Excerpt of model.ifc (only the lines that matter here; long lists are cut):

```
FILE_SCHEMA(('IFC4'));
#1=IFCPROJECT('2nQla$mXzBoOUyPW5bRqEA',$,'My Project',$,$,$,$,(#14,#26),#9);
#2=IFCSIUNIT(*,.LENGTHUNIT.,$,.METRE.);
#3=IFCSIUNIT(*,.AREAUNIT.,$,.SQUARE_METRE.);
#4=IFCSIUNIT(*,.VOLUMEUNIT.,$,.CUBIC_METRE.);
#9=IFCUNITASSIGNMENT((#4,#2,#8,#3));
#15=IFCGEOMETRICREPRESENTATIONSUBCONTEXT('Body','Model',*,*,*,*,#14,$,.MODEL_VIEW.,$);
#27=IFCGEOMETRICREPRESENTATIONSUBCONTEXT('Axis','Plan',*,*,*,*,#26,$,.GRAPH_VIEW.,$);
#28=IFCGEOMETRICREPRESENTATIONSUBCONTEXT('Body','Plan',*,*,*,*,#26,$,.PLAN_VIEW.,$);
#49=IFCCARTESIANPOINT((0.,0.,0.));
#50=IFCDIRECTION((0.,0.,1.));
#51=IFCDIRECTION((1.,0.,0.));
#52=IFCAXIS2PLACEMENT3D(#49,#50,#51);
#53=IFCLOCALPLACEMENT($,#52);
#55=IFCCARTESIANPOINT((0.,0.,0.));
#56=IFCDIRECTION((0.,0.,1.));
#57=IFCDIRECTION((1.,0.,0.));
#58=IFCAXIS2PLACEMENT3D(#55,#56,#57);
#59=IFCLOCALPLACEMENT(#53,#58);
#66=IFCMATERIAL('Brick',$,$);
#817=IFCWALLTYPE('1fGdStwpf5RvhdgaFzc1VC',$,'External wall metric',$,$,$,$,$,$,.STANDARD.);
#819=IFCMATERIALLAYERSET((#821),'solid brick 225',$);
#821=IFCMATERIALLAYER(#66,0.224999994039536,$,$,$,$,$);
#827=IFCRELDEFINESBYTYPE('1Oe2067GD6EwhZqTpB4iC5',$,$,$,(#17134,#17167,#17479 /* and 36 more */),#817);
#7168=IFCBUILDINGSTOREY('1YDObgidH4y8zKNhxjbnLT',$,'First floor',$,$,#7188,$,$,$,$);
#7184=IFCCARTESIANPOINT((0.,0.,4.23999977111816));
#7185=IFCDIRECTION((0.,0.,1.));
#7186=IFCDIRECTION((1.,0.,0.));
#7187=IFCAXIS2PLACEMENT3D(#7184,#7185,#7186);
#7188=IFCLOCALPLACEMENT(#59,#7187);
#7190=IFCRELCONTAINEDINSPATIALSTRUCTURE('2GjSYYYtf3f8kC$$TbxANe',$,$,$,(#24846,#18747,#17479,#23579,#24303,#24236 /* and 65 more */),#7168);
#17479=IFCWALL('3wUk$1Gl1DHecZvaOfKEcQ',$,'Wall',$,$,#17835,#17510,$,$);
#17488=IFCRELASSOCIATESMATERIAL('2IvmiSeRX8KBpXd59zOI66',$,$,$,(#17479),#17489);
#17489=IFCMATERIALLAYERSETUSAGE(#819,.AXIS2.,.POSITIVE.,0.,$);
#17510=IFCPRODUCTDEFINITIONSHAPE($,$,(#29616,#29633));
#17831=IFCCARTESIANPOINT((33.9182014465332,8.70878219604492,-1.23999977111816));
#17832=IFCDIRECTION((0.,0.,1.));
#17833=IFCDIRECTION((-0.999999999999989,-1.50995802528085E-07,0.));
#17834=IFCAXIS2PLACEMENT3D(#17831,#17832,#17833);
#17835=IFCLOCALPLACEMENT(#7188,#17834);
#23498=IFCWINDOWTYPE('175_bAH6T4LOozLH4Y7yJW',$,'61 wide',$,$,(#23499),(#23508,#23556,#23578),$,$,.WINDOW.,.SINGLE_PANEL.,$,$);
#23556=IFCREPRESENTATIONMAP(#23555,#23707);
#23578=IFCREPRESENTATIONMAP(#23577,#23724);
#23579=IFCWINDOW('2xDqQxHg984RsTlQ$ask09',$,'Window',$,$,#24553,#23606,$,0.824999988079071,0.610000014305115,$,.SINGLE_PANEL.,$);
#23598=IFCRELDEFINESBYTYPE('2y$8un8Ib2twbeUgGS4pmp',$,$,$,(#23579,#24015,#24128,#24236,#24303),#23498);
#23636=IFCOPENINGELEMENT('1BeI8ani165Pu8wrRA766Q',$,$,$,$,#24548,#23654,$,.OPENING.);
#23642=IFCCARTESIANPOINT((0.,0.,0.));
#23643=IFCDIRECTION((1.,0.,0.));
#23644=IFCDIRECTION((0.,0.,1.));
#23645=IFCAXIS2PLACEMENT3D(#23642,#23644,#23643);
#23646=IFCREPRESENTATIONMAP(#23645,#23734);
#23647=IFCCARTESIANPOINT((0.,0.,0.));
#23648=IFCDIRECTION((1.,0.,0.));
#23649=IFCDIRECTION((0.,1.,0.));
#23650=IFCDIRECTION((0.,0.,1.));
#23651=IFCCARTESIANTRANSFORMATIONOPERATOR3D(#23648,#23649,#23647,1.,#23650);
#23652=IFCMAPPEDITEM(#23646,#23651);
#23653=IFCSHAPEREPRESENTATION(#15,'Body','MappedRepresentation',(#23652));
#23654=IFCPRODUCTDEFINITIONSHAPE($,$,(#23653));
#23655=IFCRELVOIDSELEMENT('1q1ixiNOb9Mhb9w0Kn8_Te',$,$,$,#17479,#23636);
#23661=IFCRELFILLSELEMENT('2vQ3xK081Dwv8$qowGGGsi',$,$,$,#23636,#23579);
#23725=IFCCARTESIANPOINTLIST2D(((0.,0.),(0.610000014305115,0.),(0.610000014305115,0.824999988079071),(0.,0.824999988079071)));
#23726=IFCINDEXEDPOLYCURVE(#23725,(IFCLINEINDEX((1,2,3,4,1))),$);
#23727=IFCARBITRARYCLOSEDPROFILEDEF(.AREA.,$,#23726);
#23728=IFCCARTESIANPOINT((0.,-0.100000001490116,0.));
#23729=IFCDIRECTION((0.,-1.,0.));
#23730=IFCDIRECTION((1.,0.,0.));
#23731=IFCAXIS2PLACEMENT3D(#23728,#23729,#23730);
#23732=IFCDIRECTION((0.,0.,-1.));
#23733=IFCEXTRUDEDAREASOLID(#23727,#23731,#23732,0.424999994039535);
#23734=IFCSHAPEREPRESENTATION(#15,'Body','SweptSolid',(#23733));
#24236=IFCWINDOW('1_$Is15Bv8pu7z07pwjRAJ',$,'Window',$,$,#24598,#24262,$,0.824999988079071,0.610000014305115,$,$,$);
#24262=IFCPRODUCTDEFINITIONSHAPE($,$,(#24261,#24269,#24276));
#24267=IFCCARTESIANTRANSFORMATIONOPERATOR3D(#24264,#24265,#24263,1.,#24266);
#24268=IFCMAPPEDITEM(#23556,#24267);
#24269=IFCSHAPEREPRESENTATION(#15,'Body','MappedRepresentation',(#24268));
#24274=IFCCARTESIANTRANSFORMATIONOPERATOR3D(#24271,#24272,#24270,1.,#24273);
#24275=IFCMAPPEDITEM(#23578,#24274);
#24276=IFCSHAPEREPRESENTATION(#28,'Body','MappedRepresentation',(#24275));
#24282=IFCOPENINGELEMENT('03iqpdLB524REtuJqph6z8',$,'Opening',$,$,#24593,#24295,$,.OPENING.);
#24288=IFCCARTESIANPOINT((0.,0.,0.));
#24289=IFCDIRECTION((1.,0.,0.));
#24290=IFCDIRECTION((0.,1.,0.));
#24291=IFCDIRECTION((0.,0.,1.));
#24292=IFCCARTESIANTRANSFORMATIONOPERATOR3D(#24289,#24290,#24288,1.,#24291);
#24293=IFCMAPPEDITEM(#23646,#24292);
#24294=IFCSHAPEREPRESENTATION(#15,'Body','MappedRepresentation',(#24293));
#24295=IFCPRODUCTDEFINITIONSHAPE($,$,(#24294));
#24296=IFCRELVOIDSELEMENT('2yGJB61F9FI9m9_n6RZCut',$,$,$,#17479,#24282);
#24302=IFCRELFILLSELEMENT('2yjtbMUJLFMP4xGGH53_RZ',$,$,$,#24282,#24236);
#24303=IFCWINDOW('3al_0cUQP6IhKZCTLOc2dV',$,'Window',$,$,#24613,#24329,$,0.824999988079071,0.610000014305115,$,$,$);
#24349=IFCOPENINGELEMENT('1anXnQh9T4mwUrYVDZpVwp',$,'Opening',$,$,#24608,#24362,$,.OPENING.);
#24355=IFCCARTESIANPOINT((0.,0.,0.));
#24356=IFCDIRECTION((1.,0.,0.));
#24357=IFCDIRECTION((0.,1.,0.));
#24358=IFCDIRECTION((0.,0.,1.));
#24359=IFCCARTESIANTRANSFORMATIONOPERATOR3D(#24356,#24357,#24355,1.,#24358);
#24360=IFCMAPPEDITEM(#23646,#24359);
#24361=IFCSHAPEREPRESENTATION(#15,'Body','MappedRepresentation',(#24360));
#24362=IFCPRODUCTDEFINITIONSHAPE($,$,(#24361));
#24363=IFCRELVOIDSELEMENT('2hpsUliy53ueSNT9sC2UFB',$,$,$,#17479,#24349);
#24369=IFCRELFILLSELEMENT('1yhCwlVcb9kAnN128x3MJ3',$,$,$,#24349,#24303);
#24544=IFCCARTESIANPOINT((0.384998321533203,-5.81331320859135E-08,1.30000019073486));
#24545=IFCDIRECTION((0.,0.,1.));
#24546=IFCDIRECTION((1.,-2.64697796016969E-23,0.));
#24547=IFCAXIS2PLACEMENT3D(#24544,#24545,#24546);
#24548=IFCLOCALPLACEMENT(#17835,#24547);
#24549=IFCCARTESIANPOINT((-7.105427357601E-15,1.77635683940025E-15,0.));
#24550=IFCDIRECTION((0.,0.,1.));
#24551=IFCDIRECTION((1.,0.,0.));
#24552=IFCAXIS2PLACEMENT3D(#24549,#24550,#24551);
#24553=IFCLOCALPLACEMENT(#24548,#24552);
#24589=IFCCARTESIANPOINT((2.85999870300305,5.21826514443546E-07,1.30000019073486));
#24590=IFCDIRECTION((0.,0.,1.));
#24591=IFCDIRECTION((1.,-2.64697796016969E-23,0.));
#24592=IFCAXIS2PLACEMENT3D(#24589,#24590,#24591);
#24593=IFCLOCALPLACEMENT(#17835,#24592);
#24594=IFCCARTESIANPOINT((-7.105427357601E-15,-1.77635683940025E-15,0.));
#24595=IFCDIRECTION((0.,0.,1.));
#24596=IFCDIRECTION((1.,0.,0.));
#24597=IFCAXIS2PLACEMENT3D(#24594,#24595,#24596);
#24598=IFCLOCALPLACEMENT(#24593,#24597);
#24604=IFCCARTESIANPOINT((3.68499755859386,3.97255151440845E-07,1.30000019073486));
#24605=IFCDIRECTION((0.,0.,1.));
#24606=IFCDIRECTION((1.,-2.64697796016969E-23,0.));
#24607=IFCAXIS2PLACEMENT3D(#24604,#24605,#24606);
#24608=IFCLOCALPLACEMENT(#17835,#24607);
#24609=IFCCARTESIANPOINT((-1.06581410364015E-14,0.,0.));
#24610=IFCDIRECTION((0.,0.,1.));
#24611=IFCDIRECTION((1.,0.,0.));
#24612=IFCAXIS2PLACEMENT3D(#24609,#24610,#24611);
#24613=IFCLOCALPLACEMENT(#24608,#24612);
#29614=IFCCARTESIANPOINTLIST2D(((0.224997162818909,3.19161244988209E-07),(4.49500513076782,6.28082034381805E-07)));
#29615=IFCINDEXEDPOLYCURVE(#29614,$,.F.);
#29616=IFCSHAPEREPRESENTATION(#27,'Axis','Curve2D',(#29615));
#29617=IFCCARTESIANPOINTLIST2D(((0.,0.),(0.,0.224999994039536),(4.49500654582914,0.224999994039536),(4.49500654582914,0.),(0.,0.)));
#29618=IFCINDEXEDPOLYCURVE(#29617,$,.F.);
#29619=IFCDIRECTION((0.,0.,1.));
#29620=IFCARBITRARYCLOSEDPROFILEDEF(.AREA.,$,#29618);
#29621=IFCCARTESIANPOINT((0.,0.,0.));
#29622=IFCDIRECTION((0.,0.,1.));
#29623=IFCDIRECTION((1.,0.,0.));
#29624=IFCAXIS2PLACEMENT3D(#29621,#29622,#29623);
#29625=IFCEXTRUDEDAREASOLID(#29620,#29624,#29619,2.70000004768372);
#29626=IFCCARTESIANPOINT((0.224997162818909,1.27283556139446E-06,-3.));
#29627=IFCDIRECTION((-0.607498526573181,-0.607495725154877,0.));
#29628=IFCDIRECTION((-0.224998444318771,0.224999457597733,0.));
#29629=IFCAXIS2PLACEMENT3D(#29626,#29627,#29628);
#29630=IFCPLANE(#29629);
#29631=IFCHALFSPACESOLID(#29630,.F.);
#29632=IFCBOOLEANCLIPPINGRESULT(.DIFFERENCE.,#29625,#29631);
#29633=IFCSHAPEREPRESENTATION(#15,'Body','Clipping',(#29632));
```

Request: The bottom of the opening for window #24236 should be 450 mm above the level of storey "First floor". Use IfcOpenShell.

```python
import numpy as np
import ifcopenshell
import ifcopenshell.api.geometry
import ifcopenshell.geom
import ifcopenshell.util.element
import ifcopenshell.util.placement
import ifcopenshell.util.shape
import ifcopenshell.util.unit

model = ifcopenshell.open("model.ifc")
unit_scale = ifcopenshell.util.unit.calculate_unit_scale(model)

window = model.by_guid("1_$Is15Bv8pu7z07pwjRAJ")
opening = window.FillsVoids[0].RelatingOpeningElement
storey = ifcopenshell.util.element.get_container(window, ifc_class="IfcBuildingStorey")
level = ifcopenshell.util.placement.get_local_placement(storey.ObjectPlacement)[2, 3]

# The opening's origin need not be at the sill, so measure its lowest point.
shape = ifcopenshell.geom.create_shape(ifcopenshell.geom.settings(), opening)
bottom = ifcopenshell.util.shape.get_shape_bottom_elevation(shape, shape.geometry) / unit_scale
dz = level + 0.45 - bottom

shift = np.array([0.0, 0.0, dz])
# The window is placed relative to its opening, so it follows when the opening moves.
matrix = ifcopenshell.util.placement.get_local_placement(opening.ObjectPlacement)
matrix[:3, 3] += shift
ifcopenshell.api.geometry.edit_object_placement(
    model, product=opening, matrix=matrix, is_si=False, should_transform_children=True
)

print(f"moved by {dz * unit_scale:+.3f} m")

model.write("model_v2.ifc")
```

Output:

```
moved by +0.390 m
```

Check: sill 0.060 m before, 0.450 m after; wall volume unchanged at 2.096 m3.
